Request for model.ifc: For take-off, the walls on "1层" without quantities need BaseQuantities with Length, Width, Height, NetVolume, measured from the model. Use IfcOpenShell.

First a look at what the model holds.

```python
import ifcopenshell
import ifcopenshell.util.element
import ifcopenshell.util.unit

model = ifcopenshell.open("model.ifc")
print(model.schema)
for unit_type in ("LENGTHUNIT", "AREAUNIT", "VOLUMEUNIT"):
    print(unit_type, ifcopenshell.util.unit.calculate_unit_scale(model, unit_type))
storey = next(s for s in model.by_type("IfcBuildingStorey") if s.Name == "1层")
walls = [e for e in ifcopenshell.util.element.get_decomposition(storey) if e.is_a("IfcWall")]
for e in sorted(walls, key=lambda e: e.id()):
    print(e.id(), e.is_a(), e.Name, list(ifcopenshell.util.element.get_psets(e, qtos_only=True)), sep=" | ")
```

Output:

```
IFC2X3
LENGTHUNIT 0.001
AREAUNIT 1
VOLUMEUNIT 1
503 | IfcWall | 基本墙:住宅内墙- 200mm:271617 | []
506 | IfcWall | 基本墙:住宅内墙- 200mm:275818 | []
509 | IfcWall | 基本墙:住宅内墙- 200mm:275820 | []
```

```python
import ifcopenshell
import ifcopenshell.api.pset
import ifcopenshell.geom
import ifcopenshell.util.element
import ifcopenshell.util.shape
import ifcopenshell.util.unit

model = ifcopenshell.open("model.ifc")
unit_scale = ifcopenshell.util.unit.calculate_unit_scale(model)
volume_scale = ifcopenshell.util.unit.calculate_unit_scale(model, "VOLUMEUNIT")
settings = ifcopenshell.geom.settings()

storey = next(s for s in model.by_type("IfcBuildingStorey") if s.Name == "1层")
walls = [e for e in ifcopenshell.util.element.get_decomposition(storey) if e.is_a("IfcWall")]

for e in sorted(walls, key=lambda e: e.id()):
    if ifcopenshell.util.element.get_psets(e, qtos_only=True, should_inherit=False):
        continue
    # Geometry comes back in metres, in the element's own axes.
    shape = ifcopenshell.geom.create_shape(settings, e)
    values = {
        "Length": ifcopenshell.util.shape.get_x(shape.geometry) / unit_scale,
        "Width": ifcopenshell.util.shape.get_y(shape.geometry) / unit_scale,
        "Height": ifcopenshell.util.shape.get_z(shape.geometry) / unit_scale,
        "NetVolume": ifcopenshell.util.shape.get_volume(shape.geometry) / volume_scale,
    }
    qto = ifcopenshell.api.pset.add_qto(model, product=e, name="BaseQuantities")
    ifcopenshell.api.pset.edit_qto(model, qto=qto, properties=values)
    print(e.id(), {k: round(v, 3) for k, v in values.items()})

model.write("model_updated.ifc")
```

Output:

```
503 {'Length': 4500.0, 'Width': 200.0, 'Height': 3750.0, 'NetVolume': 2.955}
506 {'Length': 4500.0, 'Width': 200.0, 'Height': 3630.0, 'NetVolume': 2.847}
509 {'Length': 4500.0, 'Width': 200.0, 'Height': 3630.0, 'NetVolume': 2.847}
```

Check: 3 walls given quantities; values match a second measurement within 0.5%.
